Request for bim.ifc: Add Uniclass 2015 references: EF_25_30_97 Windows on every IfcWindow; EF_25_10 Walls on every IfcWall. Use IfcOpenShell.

First a look at what the model holds.

```python
import ifcopenshell

model = ifcopenshell.open("bim.ifc")
print(model.schema)
print("classifications:", [c.Name for c in model.by_type("IfcClassification")])
for ifc_class in ("IfcDoor", "IfcRoof", "IfcStair", "IfcWall", "IfcWindow"):
    print(ifc_class, len(model.by_type(ifc_class)))
```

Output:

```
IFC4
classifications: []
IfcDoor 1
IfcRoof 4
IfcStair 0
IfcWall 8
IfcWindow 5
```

```python
import ifcopenshell
import ifcopenshell.api.classification

model = ifcopenshell.open("bim.ifc")

system = ifcopenshell.api.classification.add_classification(model, classification="Uniclass 2015")

codes = {
    "IfcWindow": ("EF_25_30_97", "Windows"),
    "IfcWall": ("EF_25_10", "Walls"),
}
for ifc_class, (code, name) in codes.items():
    products = model.by_type(ifc_class)
    ifcopenshell.api.classification.add_reference(
        model, products=products, classification=system, identification=code, name=name
    )
    print(code, len(products))

model.write("bim-out.ifc")
```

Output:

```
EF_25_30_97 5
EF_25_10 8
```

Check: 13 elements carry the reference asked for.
